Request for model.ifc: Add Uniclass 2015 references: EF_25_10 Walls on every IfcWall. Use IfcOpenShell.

First a look at what the model holds.

```python
import ifcopenshell

model = ifcopenshell.open("model.ifc")
print(model.schema)
print("classifications:", [c.Name for c in model.by_type("IfcClassification")])
for ifc_class in ("IfcDoor", "IfcRoof", "IfcStair", "IfcWall", "IfcWindow"):
    print(ifc_class, len(model.by_type(ifc_class)))
```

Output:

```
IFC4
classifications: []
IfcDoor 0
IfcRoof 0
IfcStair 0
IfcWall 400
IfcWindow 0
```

```python
import ifcopenshell
import ifcopenshell.api.classification

model = ifcopenshell.open("model.ifc")

system = ifcopenshell.api.classification.add_classification(model, classification="Uniclass 2015")

codes = {
    "IfcWall": ("EF_25_10", "Walls"),
}
for ifc_class, (code, name) in codes.items():
    products = model.by_type(ifc_class)
    ifcopenshell.api.classification.add_reference(
        model, products=products, classification=system, identification=code, name=name
    )
    print(code, len(products))

model.write("model_updated.ifc")
```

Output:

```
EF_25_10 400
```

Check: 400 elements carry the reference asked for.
